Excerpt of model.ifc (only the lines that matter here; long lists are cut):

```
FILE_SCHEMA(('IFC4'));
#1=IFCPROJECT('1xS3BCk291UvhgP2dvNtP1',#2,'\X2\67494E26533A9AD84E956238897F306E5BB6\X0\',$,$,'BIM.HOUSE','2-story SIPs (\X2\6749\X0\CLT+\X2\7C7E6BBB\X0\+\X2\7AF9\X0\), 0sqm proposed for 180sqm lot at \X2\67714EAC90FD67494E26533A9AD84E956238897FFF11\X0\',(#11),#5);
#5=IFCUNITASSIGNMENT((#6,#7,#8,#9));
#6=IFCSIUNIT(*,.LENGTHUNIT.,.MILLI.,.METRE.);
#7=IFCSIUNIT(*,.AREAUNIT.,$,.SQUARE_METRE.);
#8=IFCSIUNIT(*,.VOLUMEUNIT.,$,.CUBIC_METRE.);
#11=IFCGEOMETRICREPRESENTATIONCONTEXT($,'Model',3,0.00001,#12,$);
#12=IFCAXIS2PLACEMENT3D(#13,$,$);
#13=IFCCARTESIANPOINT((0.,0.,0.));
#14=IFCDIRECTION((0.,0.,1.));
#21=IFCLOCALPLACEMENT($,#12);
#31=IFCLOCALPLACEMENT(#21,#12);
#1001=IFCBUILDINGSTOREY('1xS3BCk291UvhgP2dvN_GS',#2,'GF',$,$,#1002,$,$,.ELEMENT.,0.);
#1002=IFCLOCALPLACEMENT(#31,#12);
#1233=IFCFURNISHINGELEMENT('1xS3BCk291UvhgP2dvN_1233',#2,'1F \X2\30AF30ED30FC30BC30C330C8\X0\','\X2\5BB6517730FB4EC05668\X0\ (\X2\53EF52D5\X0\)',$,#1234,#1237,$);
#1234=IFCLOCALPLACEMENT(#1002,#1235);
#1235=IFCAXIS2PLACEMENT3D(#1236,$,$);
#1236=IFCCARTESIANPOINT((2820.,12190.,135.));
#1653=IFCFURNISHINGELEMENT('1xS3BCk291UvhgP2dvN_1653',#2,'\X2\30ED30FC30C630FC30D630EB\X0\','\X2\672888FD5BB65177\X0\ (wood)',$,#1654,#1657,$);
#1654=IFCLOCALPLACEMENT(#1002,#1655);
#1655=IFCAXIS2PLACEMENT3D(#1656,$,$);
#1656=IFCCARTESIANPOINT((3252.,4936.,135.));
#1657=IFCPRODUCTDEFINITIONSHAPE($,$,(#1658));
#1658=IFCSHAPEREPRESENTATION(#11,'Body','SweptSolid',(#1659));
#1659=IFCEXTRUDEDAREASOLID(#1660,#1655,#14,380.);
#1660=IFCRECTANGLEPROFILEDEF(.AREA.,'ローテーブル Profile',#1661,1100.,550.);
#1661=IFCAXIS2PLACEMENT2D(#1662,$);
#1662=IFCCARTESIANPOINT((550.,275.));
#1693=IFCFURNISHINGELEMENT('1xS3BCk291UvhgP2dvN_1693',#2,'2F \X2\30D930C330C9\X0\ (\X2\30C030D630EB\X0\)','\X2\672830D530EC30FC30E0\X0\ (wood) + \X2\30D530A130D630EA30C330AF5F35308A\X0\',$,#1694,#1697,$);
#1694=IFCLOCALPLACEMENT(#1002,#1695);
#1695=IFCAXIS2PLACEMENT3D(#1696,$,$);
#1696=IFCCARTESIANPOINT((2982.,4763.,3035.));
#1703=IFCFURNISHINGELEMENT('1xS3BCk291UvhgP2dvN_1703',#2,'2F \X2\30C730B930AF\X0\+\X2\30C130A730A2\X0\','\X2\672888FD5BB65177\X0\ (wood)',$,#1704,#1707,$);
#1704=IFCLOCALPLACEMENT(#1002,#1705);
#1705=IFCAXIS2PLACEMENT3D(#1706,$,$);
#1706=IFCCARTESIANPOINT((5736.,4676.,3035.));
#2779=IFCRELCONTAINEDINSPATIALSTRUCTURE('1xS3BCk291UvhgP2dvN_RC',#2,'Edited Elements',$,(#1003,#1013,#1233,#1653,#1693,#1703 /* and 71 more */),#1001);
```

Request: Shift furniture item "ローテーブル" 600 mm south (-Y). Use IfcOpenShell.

```python
import ifcopenshell
import ifcopenshell.api.geometry
import ifcopenshell.util.placement

model = ifcopenshell.open("model.ifc")

item = model.by_guid("1xS3BCk291UvhgP2dvN_1653")
matrix = ifcopenshell.util.placement.get_local_placement(item.ObjectPlacement)
matrix[1, 3] -= 600.0
ifcopenshell.api.geometry.edit_object_placement(model, product=item, matrix=matrix, is_si=False)

print(ifcopenshell.util.placement.get_local_placement(item.ObjectPlacement).round(3) + 0.0)

model.write("model_rev.ifc")
```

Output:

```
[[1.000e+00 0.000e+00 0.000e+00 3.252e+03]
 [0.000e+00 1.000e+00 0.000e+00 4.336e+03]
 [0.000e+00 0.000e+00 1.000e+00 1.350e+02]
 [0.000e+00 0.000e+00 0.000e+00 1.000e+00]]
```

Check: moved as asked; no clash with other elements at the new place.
